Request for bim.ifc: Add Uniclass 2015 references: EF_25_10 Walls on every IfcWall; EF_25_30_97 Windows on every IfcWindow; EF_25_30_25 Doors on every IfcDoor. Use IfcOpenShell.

First a look at what the model holds.

```python
import ifcopenshell

model = ifcopenshell.open("bim.ifc")
print(model.schema)
print("classifications:", [c.Name for c in model.by_type("IfcClassification")])
for ifc_class in ("IfcDoor", "IfcRoof", "IfcStair", "IfcWall", "IfcWindow"):
    print(ifc_class, len(model.by_type(ifc_class)))
```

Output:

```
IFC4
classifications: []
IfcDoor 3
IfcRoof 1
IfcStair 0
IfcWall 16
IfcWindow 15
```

```python
import ifcopenshell
import ifcopenshell.api.classification

model = ifcopenshell.open("bim.ifc")

system = ifcopenshell.api.classification.add_classification(model, classification="Uniclass 2015")

codes = {
    "IfcWall": ("EF_25_10", "Walls"),
    "IfcWindow": ("EF_25_30_97", "Windows"),
    "IfcDoor": ("EF_25_30_25", "Doors"),
}
for ifc_class, (code, name) in codes.items():
    products = model.by_type(ifc_class)
    ifcopenshell.api.classification.add_reference(
        model, products=products, classification=system, identification=code, name=name
    )
    print(code, len(products))

model.write("bim_edited.ifc")
```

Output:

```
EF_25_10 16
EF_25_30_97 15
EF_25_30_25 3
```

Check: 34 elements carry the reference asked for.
